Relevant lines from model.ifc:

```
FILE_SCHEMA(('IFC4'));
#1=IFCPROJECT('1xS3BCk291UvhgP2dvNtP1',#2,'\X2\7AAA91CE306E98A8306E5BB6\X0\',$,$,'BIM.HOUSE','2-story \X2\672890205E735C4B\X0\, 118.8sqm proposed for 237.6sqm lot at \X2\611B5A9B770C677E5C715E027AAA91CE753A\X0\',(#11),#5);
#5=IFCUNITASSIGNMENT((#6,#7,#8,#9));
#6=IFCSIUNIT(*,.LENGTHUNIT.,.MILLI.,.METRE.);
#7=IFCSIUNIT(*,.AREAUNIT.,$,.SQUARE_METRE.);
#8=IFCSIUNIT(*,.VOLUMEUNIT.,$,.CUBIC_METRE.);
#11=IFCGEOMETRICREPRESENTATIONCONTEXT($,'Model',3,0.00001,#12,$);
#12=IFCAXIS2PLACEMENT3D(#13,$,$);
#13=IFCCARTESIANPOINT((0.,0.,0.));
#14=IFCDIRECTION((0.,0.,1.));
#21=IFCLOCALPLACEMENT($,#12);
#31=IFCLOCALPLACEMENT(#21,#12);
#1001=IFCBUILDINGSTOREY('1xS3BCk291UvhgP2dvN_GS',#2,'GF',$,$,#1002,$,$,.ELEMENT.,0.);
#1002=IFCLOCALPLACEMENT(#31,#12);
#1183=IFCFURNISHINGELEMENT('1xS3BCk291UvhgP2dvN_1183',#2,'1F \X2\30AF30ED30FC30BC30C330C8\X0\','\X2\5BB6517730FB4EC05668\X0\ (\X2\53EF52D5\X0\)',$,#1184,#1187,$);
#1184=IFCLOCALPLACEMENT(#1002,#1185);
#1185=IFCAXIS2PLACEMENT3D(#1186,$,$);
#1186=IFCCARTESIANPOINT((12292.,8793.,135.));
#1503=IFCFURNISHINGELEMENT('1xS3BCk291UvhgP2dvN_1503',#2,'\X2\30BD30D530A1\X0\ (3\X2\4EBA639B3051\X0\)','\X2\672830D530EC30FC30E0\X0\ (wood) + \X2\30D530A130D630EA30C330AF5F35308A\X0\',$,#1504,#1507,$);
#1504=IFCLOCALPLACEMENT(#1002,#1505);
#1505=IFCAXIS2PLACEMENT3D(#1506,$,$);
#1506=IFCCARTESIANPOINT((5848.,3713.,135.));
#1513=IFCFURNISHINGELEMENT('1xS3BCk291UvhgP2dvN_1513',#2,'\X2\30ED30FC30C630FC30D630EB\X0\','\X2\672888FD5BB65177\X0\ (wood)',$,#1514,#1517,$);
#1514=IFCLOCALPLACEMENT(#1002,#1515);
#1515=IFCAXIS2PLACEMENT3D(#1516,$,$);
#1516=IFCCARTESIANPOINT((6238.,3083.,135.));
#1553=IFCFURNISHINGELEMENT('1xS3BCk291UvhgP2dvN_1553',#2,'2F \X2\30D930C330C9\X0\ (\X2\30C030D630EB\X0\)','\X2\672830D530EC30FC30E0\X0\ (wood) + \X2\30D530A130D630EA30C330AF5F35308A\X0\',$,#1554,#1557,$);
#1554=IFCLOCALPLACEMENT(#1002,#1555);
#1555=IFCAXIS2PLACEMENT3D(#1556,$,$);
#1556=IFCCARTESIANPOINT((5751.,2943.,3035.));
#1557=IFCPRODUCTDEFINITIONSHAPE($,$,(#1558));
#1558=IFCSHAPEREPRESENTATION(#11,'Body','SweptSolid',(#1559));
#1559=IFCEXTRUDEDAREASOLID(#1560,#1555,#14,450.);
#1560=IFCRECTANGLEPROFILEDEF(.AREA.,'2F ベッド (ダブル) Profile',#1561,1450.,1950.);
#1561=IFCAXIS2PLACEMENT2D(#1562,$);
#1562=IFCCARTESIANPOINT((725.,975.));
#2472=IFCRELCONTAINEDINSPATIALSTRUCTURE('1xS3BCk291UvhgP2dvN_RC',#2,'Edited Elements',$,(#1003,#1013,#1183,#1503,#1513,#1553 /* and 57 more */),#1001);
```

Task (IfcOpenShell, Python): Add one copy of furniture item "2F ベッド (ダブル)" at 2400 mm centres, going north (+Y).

```python
import numpy as np
import ifcopenshell
import ifcopenshell.api.geometry
import ifcopenshell.api.root
import ifcopenshell.util.element
import ifcopenshell.util.placement
import ifcopenshell.util.unit

model = ifcopenshell.open("model.ifc")
unit_scale = ifcopenshell.util.unit.calculate_unit_scale(model)


def reuse_history(source, copy):
    """copy_class also copies each property set's owner history, people and application; keep the originals."""
    for rel in copy.IsDefinedBy:
        if rel.is_a("IfcRelDefinesByProperties") and (history := rel.RelatingPropertyDefinition.OwnerHistory):
            rel.RelatingPropertyDefinition.OwnerHistory = source.OwnerHistory
            ifcopenshell.util.element.remove_deep2(model, history)


source = model.by_id(1553)
base = ifcopenshell.util.placement.get_local_placement(source.ObjectPlacement)
step = np.array([0.0, 1.0, 0.0]) * 2.4 / unit_scale

for i in range(1, 2):
    copy = ifcopenshell.api.root.copy_class(model, product=source)
    copy.Representation = ifcopenshell.util.element.copy_deep(
        model, source.Representation, exclude=["IfcGeometricRepresentationContext", "IfcRepresentationMap"]
    )
    reuse_history(source, copy)
    matrix = base.copy()
    matrix[:3, 3] += i * step
    print("added at", matrix[:3, 3].round(3) + 0.0)
    ifcopenshell.api.geometry.edit_object_placement(model, product=copy, matrix=matrix, is_si=False)

model.write("model_v2.ifc")
```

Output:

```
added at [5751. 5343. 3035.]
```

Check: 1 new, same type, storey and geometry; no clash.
